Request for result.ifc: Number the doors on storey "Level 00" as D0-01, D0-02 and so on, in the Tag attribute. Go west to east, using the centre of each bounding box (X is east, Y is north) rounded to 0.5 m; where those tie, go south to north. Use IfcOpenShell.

First a look at what the model holds.

```python
import ifcopenshell
import ifcopenshell.util.element
import ifcopenshell.util.placement

model = ifcopenshell.open("result.ifc")
print(model.schema)
storey = next(s for s in model.by_type("IfcBuildingStorey") if s.Name == "Level 00")
doors = [e for e in ifcopenshell.util.element.get_decomposition(storey) if e.is_a("IfcDoor")]
for e in sorted(doors, key=lambda e: e.id()):
    origin = ifcopenshell.util.placement.get_local_placement(e.ObjectPlacement)[:3, 3]
    print(e.id(), e.Tag, e.Name, origin.round(2) + 0.0, sep=" | ")
```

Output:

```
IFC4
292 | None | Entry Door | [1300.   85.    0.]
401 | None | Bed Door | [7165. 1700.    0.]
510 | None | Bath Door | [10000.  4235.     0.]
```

```python
import ifcopenshell
import ifcopenshell.geom
import ifcopenshell.util.element
import ifcopenshell.util.shape

model = ifcopenshell.open("result.ifc")
settings = ifcopenshell.geom.settings()
settings.set("use-world-coords", True)


def centre(element):
    shape = ifcopenshell.geom.create_shape(settings, element)
    return ifcopenshell.util.shape.get_bbox_centroid(shape.geometry)


storey = next(s for s in model.by_type("IfcBuildingStorey") if s.Name == "Level 00")
doors = [e for e in ifcopenshell.util.element.get_decomposition(storey) if e.is_a("IfcDoor")]

# Insertion points can sit at a corner or the storey origin, so sort by the geometry (in metres).
centres = {e: centre(e) for e in doors}
doors.sort(key=lambda e: (round(centres[e][0] / 0.5), centres[e][1]))

for i, e in enumerate(doors, start=1):
    number = f"D0-{i:02d}"
    e.Tag = number
    print(e.id(), number)

model.write("result_updated.ifc")
```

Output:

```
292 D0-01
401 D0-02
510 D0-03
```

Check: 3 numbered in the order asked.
